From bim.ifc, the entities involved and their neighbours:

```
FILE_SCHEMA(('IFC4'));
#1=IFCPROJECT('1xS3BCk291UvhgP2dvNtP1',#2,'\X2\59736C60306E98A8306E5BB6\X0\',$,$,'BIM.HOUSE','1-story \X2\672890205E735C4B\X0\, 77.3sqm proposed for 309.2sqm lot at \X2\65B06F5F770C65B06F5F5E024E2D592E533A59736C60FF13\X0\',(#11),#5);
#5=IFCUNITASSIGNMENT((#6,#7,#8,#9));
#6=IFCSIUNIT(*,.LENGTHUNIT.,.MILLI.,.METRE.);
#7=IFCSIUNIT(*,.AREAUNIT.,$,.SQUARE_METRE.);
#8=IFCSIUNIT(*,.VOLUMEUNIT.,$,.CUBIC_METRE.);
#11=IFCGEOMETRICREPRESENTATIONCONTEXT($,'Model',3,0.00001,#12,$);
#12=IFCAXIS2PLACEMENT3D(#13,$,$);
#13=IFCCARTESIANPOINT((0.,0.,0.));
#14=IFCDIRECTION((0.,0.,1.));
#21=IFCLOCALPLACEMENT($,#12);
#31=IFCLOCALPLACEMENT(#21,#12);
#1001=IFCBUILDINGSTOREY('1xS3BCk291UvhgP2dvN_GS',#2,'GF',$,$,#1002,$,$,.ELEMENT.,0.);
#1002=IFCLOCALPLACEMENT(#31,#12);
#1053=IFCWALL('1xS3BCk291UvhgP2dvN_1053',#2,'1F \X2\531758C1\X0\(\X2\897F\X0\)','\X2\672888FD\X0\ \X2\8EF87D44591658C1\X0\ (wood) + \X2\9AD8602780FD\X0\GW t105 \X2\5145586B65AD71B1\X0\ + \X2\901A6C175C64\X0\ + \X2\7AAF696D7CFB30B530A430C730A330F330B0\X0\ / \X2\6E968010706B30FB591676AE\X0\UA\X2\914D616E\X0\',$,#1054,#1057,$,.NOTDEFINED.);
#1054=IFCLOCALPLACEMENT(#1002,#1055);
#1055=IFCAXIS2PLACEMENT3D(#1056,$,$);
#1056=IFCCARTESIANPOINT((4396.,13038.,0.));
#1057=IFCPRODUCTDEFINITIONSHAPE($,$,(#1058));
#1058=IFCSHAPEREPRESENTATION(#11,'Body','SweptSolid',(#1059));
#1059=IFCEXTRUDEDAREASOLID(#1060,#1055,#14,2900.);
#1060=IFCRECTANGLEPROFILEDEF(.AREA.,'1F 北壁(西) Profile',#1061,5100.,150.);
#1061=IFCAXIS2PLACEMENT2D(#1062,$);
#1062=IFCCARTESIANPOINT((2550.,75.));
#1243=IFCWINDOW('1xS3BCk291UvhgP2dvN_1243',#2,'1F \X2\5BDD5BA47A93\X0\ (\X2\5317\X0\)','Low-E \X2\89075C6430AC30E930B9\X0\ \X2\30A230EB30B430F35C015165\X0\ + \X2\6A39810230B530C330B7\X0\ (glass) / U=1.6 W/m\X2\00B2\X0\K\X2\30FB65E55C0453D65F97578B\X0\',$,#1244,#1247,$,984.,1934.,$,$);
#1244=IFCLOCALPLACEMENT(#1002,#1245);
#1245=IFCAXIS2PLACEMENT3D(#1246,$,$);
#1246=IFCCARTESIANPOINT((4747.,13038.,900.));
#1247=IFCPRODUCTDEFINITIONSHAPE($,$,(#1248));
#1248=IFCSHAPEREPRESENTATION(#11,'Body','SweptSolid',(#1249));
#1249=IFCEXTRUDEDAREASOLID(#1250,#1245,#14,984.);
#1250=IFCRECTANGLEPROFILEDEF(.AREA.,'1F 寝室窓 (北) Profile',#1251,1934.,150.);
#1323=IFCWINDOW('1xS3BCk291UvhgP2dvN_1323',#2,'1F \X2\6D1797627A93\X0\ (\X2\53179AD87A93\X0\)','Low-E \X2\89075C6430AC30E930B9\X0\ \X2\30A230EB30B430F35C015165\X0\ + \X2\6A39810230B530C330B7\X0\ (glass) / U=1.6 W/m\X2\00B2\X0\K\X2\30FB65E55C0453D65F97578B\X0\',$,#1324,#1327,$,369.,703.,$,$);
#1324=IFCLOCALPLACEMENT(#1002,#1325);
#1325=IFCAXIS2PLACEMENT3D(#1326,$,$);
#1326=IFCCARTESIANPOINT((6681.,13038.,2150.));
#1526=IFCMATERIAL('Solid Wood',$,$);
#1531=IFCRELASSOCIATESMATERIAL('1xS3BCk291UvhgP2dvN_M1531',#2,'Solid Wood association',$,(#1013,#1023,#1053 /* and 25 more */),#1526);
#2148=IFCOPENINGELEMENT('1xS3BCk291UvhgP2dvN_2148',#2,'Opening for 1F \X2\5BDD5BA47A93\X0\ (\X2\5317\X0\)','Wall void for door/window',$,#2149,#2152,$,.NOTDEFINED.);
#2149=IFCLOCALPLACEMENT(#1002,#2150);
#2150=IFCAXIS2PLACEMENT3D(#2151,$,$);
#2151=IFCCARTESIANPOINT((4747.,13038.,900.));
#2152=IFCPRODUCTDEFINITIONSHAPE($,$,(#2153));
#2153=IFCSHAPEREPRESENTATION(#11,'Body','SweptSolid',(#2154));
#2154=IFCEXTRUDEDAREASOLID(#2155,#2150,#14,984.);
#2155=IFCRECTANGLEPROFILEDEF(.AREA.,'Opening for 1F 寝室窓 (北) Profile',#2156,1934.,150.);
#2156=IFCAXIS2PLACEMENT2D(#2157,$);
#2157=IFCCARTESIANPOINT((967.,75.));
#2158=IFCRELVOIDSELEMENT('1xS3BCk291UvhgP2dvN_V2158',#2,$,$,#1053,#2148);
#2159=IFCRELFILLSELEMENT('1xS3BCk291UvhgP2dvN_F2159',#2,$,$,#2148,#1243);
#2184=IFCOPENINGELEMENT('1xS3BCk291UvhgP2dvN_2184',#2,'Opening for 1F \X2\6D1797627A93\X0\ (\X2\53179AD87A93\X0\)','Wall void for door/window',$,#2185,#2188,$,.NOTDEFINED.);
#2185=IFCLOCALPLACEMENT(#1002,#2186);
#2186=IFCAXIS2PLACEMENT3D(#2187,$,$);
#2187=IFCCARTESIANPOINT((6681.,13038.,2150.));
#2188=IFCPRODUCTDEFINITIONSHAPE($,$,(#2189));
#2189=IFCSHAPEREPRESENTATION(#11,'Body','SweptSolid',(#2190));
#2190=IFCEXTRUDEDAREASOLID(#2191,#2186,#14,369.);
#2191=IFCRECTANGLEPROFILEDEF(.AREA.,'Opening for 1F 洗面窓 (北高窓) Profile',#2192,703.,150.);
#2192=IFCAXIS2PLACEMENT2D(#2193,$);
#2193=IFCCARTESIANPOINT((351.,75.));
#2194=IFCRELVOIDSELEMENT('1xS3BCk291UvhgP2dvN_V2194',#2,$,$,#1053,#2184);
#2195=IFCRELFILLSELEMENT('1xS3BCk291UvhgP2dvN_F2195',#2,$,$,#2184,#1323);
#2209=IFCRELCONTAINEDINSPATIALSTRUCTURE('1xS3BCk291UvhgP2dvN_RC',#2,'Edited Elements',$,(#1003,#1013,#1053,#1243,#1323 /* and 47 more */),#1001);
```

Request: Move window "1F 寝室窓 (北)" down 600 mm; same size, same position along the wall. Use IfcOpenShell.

```python
import numpy as np
import ifcopenshell
import ifcopenshell.api.geometry
import ifcopenshell.util.placement
import ifcopenshell.util.unit

model = ifcopenshell.open("bim.ifc")
unit_scale = ifcopenshell.util.unit.calculate_unit_scale(model)

window = model.by_guid("1xS3BCk291UvhgP2dvN_1243")
opening = window.FillsVoids[0].RelatingOpeningElement
dz = -0.6 / unit_scale

shift = np.array([0.0, 0.0, dz])
# The window is not placed relative to its opening, so move both.
for product in (opening, window):
    matrix = ifcopenshell.util.placement.get_local_placement(product.ObjectPlacement)
    matrix[:3, 3] += shift
    ifcopenshell.api.geometry.edit_object_placement(model, product=product, matrix=matrix, is_si=False)

print(f"moved by {dz * unit_scale:+.3f} m")

model.write("bim-out.ifc")
```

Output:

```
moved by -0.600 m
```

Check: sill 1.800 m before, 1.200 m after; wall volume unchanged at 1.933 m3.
